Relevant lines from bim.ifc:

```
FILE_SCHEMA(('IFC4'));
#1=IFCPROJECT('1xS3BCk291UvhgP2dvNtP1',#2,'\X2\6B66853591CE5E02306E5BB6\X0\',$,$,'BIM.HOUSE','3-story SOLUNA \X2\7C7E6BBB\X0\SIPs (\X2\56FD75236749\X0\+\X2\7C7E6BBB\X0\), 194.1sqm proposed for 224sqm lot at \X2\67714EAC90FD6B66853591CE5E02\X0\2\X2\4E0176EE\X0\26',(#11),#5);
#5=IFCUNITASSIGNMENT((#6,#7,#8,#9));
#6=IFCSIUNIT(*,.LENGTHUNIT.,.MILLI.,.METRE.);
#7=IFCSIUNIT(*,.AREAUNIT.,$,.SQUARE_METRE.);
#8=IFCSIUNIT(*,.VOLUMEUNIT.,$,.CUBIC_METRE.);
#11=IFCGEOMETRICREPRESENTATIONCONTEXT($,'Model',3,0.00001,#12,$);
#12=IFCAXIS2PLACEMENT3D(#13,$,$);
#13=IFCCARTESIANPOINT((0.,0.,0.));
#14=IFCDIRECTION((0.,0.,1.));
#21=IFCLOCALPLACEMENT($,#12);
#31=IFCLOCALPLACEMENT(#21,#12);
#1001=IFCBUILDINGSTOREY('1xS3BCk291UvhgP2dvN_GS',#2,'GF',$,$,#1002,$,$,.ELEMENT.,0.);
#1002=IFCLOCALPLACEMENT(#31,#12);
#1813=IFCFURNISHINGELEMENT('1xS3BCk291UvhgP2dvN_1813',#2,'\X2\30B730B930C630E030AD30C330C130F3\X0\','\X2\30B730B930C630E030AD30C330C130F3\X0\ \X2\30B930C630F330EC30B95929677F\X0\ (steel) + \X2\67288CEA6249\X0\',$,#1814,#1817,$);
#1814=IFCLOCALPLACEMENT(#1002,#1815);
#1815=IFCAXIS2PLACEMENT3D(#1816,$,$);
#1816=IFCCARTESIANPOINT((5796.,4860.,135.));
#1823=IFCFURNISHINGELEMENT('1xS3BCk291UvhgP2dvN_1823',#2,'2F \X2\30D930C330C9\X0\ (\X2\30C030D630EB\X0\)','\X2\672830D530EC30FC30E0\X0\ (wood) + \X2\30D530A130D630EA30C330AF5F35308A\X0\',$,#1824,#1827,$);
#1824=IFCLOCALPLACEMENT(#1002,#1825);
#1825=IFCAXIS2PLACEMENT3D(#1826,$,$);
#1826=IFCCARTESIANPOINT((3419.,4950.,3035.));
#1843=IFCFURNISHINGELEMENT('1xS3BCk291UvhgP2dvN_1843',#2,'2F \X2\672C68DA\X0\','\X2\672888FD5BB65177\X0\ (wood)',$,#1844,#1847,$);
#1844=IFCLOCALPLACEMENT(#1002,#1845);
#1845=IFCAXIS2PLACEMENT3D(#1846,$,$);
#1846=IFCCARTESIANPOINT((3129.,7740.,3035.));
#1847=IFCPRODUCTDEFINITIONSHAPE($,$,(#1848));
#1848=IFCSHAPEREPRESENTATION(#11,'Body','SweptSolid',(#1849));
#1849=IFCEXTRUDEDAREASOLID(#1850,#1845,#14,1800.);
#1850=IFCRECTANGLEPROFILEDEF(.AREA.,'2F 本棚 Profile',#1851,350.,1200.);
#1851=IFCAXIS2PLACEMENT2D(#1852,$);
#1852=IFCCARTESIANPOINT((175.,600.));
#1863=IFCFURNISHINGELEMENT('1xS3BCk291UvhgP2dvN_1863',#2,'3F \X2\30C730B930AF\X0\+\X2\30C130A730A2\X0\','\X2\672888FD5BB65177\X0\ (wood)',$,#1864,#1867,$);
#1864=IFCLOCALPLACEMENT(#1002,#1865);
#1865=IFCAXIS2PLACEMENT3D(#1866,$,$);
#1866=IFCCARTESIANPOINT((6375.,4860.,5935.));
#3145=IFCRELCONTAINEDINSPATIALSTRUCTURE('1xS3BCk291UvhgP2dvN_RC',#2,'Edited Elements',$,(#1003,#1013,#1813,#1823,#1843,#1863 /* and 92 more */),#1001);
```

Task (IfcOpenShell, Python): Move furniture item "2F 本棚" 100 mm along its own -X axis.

```python
import ifcopenshell
import ifcopenshell.api.geometry
import ifcopenshell.util.placement
import ifcopenshell.util.unit

model = ifcopenshell.open("bim.ifc")
unit_scale = ifcopenshell.util.unit.calculate_unit_scale(model)

item = model.by_guid("1xS3BCk291UvhgP2dvN_1843")
matrix = ifcopenshell.util.placement.get_local_placement(item.ObjectPlacement)
matrix[:3, 3] -= matrix[:3, 0] * 0.1 / unit_scale
ifcopenshell.api.geometry.edit_object_placement(model, product=item, matrix=matrix, is_si=False)

print(ifcopenshell.util.placement.get_local_placement(item.ObjectPlacement).round(3) + 0.0)

model.write("bim_v2.ifc")
```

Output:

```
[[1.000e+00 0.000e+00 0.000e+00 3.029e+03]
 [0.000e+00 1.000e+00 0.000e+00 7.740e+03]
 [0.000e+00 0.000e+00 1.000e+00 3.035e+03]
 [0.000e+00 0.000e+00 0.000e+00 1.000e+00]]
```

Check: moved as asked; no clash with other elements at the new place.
